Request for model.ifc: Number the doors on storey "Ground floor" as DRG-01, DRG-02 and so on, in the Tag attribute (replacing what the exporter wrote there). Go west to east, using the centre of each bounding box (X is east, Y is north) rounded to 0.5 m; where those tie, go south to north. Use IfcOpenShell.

First a look at what the model holds.

```python
import ifcopenshell
import ifcopenshell.util.element
import ifcopenshell.util.placement

model = ifcopenshell.open("model.ifc")
print(model.schema)
storey = next(s for s in model.by_type("IfcBuildingStorey") if s.Name == "Ground floor")
doors = [e for e in ifcopenshell.util.element.get_decomposition(storey) if e.is_a("IfcDoor")]
for e in sorted(doors, key=lambda e: e.id()):
    origin = ifcopenshell.util.placement.get_local_placement(e.ObjectPlacement)[:3, 3]
    print(e.id(), e.Tag, e.Name, origin.round(2) + 0.0, sep=" | ")
```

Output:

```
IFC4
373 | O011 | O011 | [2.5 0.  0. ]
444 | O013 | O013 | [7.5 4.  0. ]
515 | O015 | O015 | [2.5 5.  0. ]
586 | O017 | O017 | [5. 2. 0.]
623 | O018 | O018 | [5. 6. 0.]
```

```python
import ifcopenshell
import ifcopenshell.geom
import ifcopenshell.util.element
import ifcopenshell.util.shape

model = ifcopenshell.open("model.ifc")
settings = ifcopenshell.geom.settings()
settings.set("use-world-coords", True)


def centre(element):
    shape = ifcopenshell.geom.create_shape(settings, element)
    return ifcopenshell.util.shape.get_bbox_centroid(shape.geometry)


storey = next(s for s in model.by_type("IfcBuildingStorey") if s.Name == "Ground floor")
doors = [e for e in ifcopenshell.util.element.get_decomposition(storey) if e.is_a("IfcDoor")]

# Insertion points can sit at a corner or the storey origin, so sort by the geometry (in metres).
centres = {e: centre(e) for e in doors}
doors.sort(key=lambda e: (round(centres[e][0] / 0.5), centres[e][1]))

for i, e in enumerate(doors, start=1):
    number = f"DRG-{i:02d}"
    e.Tag = number
    print(e.id(), number)

model.write("model_updated.ifc")
```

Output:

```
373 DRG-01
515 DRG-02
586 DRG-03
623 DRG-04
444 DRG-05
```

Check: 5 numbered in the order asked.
